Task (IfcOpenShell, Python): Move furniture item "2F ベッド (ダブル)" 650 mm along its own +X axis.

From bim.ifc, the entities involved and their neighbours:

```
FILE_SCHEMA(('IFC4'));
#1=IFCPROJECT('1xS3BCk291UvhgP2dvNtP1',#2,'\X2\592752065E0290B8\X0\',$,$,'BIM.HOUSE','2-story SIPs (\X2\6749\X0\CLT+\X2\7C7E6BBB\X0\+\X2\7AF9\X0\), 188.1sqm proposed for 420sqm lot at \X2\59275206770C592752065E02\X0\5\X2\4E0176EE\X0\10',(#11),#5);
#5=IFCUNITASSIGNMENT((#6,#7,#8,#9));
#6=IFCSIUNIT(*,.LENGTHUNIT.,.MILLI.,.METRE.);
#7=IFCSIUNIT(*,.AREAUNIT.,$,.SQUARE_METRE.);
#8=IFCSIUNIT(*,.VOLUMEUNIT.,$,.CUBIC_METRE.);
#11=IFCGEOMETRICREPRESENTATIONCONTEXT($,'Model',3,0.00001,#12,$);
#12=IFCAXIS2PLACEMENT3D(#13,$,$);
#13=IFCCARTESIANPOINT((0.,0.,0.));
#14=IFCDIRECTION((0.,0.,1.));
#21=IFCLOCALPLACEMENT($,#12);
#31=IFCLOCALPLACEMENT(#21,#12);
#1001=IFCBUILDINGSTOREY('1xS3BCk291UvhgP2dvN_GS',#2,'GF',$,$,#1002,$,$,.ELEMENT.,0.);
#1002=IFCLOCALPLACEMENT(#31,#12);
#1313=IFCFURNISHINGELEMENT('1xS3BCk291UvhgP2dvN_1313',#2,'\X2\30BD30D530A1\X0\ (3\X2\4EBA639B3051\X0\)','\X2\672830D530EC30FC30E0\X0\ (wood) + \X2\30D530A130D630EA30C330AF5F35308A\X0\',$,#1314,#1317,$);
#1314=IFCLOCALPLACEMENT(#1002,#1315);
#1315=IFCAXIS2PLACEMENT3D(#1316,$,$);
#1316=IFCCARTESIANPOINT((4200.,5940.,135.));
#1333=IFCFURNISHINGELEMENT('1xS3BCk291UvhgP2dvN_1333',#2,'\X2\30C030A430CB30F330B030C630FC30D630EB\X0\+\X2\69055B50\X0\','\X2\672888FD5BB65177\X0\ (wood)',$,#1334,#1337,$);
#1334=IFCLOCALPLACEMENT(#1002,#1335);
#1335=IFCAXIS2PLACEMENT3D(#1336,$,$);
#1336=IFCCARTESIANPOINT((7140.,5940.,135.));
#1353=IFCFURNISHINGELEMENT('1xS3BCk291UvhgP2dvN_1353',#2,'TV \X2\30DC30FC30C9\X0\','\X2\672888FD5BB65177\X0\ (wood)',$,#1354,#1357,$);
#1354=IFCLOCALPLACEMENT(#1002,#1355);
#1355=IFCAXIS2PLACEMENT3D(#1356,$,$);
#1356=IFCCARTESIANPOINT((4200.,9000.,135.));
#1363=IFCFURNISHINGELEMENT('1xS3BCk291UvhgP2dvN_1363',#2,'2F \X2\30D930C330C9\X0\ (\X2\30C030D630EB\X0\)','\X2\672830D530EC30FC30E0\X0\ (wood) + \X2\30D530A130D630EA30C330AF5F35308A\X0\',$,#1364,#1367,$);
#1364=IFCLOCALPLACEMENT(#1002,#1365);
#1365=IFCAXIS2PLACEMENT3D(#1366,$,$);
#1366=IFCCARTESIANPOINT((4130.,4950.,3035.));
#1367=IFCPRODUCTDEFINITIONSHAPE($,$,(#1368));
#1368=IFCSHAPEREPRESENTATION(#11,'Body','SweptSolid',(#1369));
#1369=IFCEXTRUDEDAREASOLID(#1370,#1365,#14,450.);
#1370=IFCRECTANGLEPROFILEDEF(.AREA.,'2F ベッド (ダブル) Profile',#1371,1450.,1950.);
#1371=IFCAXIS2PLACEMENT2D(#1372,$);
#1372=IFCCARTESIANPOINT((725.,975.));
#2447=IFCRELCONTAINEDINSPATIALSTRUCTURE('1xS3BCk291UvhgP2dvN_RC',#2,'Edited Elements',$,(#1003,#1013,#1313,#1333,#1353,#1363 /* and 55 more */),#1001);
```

```python
import ifcopenshell
import ifcopenshell.api.geometry
import ifcopenshell.util.placement
import ifcopenshell.util.unit

model = ifcopenshell.open("bim.ifc")
unit_scale = ifcopenshell.util.unit.calculate_unit_scale(model)

item = model.by_guid("1xS3BCk291UvhgP2dvN_1363")
matrix = ifcopenshell.util.placement.get_local_placement(item.ObjectPlacement)
matrix[:3, 3] += matrix[:3, 0] * 0.65 / unit_scale
ifcopenshell.api.geometry.edit_object_placement(model, product=item, matrix=matrix, is_si=False)

print(ifcopenshell.util.placement.get_local_placement(item.ObjectPlacement).round(3) + 0.0)

model.write("bim_edited.ifc")
```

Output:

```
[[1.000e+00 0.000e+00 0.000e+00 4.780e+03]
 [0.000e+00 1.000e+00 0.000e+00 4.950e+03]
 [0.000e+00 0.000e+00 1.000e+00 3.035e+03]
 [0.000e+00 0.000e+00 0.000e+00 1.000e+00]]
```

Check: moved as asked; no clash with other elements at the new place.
